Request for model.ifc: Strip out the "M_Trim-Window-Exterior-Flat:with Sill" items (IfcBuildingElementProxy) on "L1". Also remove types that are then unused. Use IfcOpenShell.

First a look at what the model holds.

```python
import ifcopenshell
import ifcopenshell.util.element

model = ifcopenshell.open("model.ifc")
print(model.schema)
storey = next(s for s in model.by_type("IfcBuildingStorey") if s.Name == "L1")
proxies = [e for e in ifcopenshell.util.element.get_decomposition(storey) if e.is_a("IfcBuildingElementProxy")]
seen = {}
for e in proxies:
    element_type = ifcopenshell.util.element.get_type(e)
    name = element_type.Name if element_type not in (None, e) else None
    seen[name] = seen.get(name, 0) + 1
for name, count in sorted(seen.items(), key=str):
    print(count, "x", name)
```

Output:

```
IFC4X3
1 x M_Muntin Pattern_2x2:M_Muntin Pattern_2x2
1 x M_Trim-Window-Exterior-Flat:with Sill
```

```python
import ifcopenshell
import ifcopenshell.api.root
import ifcopenshell.util.element

model = ifcopenshell.open("model.ifc")

storey = next(s for s in model.by_type("IfcBuildingStorey") if s.Name == "L1")
proxies = [e for e in ifcopenshell.util.element.get_decomposition(storey) if e.is_a("IfcBuildingElementProxy")]
targets = [e for e in proxies if (t := ifcopenshell.util.element.get_type(e)) not in (None, e) and t.Name == "M_Trim-Window-Exterior-Flat:with Sill"]
types = {ifcopenshell.util.element.get_type(e) for e in targets} - {None, *targets}

for e in targets:
    ifcopenshell.api.root.remove_product(model, product=e)
print(len(targets), "removed")

unused = [t for t in types if not ifcopenshell.util.element.get_types(t)]
for t in unused:
    ifcopenshell.api.root.remove_product(model, product=t)
print(len(unused), "unused types removed")

model.write("model_edited.ifc")
```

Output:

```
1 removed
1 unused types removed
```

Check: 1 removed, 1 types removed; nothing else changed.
